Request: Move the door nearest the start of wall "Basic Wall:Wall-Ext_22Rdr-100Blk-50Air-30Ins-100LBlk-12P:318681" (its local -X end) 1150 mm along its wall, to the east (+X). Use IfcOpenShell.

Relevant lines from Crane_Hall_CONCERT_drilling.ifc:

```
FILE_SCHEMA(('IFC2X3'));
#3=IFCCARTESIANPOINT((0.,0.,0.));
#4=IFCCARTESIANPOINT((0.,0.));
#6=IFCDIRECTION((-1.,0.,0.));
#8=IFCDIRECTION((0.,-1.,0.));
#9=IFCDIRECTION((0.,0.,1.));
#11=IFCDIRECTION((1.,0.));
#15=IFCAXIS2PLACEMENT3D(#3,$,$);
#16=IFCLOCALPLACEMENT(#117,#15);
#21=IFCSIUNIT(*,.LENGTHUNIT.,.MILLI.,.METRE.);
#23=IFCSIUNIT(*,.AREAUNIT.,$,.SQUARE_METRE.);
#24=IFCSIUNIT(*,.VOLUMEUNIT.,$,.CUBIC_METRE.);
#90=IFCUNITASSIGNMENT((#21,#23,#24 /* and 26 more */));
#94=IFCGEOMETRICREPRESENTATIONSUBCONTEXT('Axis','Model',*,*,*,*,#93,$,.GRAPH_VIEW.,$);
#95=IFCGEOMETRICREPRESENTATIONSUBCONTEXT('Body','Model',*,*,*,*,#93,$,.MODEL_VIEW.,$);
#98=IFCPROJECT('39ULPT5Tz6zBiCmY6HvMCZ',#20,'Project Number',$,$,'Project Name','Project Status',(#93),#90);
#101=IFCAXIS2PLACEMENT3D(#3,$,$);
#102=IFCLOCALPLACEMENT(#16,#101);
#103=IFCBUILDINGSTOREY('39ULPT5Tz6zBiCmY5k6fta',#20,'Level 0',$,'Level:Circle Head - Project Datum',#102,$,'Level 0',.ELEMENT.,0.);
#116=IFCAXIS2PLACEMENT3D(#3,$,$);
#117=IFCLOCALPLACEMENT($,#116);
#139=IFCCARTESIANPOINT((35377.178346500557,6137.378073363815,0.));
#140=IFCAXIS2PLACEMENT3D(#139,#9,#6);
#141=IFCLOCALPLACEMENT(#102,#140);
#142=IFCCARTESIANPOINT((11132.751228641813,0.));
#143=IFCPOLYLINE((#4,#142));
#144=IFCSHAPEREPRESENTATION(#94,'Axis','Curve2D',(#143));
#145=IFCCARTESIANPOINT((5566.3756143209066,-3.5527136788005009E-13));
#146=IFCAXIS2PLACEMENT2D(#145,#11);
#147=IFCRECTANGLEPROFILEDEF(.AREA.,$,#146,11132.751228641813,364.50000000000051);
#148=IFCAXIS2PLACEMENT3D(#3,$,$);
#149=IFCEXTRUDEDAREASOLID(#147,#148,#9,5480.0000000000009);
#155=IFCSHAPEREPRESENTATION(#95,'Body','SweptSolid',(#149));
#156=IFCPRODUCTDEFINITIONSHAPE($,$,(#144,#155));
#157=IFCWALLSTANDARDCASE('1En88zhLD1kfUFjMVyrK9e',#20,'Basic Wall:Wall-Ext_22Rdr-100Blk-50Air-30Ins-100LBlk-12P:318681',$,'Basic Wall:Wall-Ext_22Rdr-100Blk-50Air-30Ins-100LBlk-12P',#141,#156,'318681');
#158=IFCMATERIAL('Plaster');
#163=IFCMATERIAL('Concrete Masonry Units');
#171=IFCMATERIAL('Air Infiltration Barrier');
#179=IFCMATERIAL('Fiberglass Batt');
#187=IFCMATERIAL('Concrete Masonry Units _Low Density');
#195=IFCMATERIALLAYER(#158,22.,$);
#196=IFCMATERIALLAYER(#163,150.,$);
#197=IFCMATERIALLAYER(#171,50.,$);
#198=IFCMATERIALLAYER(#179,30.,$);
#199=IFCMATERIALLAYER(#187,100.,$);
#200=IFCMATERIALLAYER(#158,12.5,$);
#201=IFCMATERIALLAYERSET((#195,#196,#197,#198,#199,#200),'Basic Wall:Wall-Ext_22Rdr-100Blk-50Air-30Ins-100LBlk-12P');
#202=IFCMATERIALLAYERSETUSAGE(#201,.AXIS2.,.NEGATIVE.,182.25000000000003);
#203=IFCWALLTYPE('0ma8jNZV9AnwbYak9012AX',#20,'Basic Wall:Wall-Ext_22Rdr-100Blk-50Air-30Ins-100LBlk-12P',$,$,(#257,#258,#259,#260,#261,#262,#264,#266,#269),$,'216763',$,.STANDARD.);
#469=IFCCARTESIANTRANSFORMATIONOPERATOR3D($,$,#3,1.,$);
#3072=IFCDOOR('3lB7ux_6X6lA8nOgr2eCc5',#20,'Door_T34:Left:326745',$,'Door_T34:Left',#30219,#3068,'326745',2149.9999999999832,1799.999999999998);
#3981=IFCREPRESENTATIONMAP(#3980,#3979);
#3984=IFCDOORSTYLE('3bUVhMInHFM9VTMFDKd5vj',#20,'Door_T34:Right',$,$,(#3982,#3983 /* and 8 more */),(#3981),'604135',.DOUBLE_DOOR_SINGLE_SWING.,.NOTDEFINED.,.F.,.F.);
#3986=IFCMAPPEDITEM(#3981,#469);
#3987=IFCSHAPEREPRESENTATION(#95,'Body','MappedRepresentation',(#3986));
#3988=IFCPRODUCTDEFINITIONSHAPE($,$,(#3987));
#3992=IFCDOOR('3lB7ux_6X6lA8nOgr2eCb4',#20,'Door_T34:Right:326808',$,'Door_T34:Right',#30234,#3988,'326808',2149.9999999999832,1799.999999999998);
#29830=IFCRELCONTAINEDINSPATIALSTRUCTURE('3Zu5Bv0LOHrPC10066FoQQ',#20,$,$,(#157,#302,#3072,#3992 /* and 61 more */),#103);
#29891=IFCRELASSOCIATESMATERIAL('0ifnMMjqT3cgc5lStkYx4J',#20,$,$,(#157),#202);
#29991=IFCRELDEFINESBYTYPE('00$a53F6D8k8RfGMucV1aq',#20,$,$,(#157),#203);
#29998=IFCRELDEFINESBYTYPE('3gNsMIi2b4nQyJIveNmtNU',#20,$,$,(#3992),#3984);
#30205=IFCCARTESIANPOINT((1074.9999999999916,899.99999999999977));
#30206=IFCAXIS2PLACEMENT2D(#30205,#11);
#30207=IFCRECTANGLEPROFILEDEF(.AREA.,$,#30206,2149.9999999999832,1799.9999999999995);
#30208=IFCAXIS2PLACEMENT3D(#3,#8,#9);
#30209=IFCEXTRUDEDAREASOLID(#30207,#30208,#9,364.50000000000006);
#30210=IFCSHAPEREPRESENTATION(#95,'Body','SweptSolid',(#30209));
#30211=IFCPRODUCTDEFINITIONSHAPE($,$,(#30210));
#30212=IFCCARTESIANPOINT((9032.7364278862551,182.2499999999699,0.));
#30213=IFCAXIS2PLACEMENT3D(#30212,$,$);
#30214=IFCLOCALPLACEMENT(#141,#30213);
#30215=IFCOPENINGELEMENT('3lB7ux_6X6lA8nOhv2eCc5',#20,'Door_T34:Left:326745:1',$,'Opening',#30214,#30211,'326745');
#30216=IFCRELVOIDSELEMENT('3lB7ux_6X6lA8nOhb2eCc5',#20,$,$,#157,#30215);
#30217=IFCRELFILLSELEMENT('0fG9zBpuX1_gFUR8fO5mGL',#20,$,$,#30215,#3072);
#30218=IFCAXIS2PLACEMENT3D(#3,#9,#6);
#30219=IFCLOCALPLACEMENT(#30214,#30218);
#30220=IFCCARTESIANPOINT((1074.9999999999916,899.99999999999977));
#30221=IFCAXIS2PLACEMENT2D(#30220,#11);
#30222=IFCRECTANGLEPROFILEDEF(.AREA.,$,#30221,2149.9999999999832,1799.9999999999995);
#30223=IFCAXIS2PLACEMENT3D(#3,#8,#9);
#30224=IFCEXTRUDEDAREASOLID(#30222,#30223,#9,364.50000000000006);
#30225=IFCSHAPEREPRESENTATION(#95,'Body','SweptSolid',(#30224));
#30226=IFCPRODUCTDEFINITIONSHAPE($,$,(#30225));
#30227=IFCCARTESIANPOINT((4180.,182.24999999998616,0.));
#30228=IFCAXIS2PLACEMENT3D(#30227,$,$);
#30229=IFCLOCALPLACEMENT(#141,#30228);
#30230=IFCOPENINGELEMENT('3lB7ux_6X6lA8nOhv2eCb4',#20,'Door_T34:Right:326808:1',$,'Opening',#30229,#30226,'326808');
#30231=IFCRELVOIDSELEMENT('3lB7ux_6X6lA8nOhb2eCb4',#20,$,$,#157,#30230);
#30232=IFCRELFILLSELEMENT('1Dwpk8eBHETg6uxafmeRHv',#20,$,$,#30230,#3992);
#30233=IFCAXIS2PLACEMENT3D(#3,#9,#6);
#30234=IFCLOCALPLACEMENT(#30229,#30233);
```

```python
import ifcopenshell
import ifcopenshell.api.geometry
import ifcopenshell.util.placement
import ifcopenshell.util.unit

model = ifcopenshell.open("Crane_Hall_CONCERT_drilling.ifc")
unit_scale = ifcopenshell.util.unit.calculate_unit_scale(model)

door = model.by_id(3992)
opening = door.FillsVoids[0].RelatingOpeningElement
wall = opening.VoidsElements[0].RelatingBuildingElement

wall_matrix = ifcopenshell.util.placement.get_local_placement(wall.ObjectPlacement)
shift = wall_matrix[:3, 0] * -1.15 / unit_scale
before = ifcopenshell.util.placement.get_local_placement(door.ObjectPlacement)[:3, 3].copy()

# The door is placed relative to its opening, so it follows when the opening moves.
matrix = ifcopenshell.util.placement.get_local_placement(opening.ObjectPlacement)
matrix[:3, 3] += shift
ifcopenshell.api.geometry.edit_object_placement(
    model, product=opening, matrix=matrix, is_si=False, should_transform_children=True
)

after = ifcopenshell.util.placement.get_local_placement(door.ObjectPlacement)[:3, 3]
print("door moved by", (after - before).round(3) + 0.0)

model.write("Crane_Hall_CONCERT_drilling_rev.ifc")
```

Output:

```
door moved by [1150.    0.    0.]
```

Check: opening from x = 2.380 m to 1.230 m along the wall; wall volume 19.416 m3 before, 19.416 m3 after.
